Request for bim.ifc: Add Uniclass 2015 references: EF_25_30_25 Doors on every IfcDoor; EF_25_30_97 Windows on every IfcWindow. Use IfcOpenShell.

First a look at what the model holds.

```python
import ifcopenshell

model = ifcopenshell.open("bim.ifc")
print(model.schema)
print("classifications:", [c.Name for c in model.by_type("IfcClassification")])
for ifc_class in ("IfcDoor", "IfcRoof", "IfcStair", "IfcWall", "IfcWindow"):
    print(ifc_class, len(model.by_type(ifc_class)))
```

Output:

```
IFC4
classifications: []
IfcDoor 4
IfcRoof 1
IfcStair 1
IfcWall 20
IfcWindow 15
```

```python
import ifcopenshell
import ifcopenshell.api.classification

model = ifcopenshell.open("bim.ifc")

system = ifcopenshell.api.classification.add_classification(model, classification="Uniclass 2015")

codes = {
    "IfcDoor": ("EF_25_30_25", "Doors"),
    "IfcWindow": ("EF_25_30_97", "Windows"),
}
for ifc_class, (code, name) in codes.items():
    products = model.by_type(ifc_class)
    ifcopenshell.api.classification.add_reference(
        model, products=products, classification=system, identification=code, name=name
    )
    print(code, len(products))

model.write("bim_updated.ifc")
```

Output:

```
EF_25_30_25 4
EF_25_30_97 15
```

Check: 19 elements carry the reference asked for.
